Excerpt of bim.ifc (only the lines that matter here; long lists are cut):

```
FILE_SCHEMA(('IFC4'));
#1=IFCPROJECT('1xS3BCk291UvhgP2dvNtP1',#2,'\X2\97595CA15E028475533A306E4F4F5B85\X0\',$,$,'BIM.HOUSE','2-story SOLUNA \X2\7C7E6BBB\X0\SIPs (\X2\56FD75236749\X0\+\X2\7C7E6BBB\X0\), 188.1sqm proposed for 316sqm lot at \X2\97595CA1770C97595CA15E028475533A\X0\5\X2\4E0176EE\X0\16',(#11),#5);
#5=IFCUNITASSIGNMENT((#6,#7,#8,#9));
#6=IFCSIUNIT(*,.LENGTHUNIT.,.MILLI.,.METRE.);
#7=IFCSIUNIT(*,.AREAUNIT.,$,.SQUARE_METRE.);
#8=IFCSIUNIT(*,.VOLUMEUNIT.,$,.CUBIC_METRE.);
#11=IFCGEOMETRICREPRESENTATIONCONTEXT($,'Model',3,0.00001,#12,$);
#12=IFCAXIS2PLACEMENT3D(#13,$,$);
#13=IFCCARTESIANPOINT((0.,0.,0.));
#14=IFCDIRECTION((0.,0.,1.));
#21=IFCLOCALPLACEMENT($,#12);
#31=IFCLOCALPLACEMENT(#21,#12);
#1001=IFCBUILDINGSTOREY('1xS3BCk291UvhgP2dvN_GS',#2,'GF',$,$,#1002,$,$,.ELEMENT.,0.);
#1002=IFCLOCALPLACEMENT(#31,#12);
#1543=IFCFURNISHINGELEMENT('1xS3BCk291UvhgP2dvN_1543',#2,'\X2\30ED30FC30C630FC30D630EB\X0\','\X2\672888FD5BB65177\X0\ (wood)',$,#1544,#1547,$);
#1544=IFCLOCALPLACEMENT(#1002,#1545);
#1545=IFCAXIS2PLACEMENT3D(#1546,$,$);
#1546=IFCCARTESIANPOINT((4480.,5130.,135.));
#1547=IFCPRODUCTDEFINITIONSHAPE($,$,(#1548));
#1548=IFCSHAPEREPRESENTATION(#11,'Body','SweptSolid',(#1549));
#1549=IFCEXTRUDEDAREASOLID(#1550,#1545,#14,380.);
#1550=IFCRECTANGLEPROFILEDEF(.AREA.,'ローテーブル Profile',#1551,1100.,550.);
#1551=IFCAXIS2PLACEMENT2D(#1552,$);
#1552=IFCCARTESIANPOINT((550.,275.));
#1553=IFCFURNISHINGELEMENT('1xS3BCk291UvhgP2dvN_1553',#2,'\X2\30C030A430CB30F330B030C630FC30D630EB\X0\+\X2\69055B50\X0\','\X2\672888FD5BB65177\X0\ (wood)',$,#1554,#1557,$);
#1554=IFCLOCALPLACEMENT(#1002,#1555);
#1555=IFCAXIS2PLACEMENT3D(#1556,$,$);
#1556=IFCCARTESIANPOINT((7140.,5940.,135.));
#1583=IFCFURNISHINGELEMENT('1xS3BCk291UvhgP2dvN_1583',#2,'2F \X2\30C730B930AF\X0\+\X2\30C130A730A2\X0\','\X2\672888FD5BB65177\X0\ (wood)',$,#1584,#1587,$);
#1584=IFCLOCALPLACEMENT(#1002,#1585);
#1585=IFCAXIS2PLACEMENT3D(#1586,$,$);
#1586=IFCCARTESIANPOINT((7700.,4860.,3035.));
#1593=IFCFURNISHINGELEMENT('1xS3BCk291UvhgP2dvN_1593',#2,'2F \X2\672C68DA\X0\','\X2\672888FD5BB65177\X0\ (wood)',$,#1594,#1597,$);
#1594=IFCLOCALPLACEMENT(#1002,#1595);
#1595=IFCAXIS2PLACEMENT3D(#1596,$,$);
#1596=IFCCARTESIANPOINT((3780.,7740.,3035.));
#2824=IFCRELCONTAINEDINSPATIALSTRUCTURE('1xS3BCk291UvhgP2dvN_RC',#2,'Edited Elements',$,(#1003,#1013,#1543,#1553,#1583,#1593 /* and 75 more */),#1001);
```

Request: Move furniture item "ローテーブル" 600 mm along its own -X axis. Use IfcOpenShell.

```python
import ifcopenshell
import ifcopenshell.api.geometry
import ifcopenshell.util.placement
import ifcopenshell.util.unit

model = ifcopenshell.open("bim.ifc")
unit_scale = ifcopenshell.util.unit.calculate_unit_scale(model)

item = model.by_guid("1xS3BCk291UvhgP2dvN_1543")
matrix = ifcopenshell.util.placement.get_local_placement(item.ObjectPlacement)
matrix[:3, 3] -= matrix[:3, 0] * 0.6 / unit_scale
ifcopenshell.api.geometry.edit_object_placement(model, product=item, matrix=matrix, is_si=False)

print(ifcopenshell.util.placement.get_local_placement(item.ObjectPlacement).round(3) + 0.0)

model.write("bim-out.ifc")
```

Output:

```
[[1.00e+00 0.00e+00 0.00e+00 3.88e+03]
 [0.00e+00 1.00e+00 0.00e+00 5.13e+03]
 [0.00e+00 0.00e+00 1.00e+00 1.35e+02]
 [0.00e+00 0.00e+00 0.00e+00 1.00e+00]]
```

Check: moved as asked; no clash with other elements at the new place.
